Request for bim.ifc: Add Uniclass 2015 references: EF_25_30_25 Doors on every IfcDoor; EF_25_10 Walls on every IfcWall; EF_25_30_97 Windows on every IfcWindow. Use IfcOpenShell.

First a look at what the model holds.

```python
import ifcopenshell

model = ifcopenshell.open("bim.ifc")
print(model.schema)
print("classifications:", [c.Name for c in model.by_type("IfcClassification")])
for ifc_class in ("IfcDoor", "IfcRoof", "IfcStair", "IfcWall", "IfcWindow"):
    print(ifc_class, len(model.by_type(ifc_class)))
```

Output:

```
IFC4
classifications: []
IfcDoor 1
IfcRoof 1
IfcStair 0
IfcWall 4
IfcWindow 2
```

```python
import ifcopenshell
import ifcopenshell.api.classification

model = ifcopenshell.open("bim.ifc")

system = ifcopenshell.api.classification.add_classification(model, classification="Uniclass 2015")

codes = {
    "IfcDoor": ("EF_25_30_25", "Doors"),
    "IfcWall": ("EF_25_10", "Walls"),
    "IfcWindow": ("EF_25_30_97", "Windows"),
}
for ifc_class, (code, name) in codes.items():
    products = model.by_type(ifc_class)
    ifcopenshell.api.classification.add_reference(
        model, products=products, classification=system, identification=code, name=name
    )
    print(code, len(products))

model.write("bim-out.ifc")
```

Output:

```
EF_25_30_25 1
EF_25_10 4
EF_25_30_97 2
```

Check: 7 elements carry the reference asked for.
